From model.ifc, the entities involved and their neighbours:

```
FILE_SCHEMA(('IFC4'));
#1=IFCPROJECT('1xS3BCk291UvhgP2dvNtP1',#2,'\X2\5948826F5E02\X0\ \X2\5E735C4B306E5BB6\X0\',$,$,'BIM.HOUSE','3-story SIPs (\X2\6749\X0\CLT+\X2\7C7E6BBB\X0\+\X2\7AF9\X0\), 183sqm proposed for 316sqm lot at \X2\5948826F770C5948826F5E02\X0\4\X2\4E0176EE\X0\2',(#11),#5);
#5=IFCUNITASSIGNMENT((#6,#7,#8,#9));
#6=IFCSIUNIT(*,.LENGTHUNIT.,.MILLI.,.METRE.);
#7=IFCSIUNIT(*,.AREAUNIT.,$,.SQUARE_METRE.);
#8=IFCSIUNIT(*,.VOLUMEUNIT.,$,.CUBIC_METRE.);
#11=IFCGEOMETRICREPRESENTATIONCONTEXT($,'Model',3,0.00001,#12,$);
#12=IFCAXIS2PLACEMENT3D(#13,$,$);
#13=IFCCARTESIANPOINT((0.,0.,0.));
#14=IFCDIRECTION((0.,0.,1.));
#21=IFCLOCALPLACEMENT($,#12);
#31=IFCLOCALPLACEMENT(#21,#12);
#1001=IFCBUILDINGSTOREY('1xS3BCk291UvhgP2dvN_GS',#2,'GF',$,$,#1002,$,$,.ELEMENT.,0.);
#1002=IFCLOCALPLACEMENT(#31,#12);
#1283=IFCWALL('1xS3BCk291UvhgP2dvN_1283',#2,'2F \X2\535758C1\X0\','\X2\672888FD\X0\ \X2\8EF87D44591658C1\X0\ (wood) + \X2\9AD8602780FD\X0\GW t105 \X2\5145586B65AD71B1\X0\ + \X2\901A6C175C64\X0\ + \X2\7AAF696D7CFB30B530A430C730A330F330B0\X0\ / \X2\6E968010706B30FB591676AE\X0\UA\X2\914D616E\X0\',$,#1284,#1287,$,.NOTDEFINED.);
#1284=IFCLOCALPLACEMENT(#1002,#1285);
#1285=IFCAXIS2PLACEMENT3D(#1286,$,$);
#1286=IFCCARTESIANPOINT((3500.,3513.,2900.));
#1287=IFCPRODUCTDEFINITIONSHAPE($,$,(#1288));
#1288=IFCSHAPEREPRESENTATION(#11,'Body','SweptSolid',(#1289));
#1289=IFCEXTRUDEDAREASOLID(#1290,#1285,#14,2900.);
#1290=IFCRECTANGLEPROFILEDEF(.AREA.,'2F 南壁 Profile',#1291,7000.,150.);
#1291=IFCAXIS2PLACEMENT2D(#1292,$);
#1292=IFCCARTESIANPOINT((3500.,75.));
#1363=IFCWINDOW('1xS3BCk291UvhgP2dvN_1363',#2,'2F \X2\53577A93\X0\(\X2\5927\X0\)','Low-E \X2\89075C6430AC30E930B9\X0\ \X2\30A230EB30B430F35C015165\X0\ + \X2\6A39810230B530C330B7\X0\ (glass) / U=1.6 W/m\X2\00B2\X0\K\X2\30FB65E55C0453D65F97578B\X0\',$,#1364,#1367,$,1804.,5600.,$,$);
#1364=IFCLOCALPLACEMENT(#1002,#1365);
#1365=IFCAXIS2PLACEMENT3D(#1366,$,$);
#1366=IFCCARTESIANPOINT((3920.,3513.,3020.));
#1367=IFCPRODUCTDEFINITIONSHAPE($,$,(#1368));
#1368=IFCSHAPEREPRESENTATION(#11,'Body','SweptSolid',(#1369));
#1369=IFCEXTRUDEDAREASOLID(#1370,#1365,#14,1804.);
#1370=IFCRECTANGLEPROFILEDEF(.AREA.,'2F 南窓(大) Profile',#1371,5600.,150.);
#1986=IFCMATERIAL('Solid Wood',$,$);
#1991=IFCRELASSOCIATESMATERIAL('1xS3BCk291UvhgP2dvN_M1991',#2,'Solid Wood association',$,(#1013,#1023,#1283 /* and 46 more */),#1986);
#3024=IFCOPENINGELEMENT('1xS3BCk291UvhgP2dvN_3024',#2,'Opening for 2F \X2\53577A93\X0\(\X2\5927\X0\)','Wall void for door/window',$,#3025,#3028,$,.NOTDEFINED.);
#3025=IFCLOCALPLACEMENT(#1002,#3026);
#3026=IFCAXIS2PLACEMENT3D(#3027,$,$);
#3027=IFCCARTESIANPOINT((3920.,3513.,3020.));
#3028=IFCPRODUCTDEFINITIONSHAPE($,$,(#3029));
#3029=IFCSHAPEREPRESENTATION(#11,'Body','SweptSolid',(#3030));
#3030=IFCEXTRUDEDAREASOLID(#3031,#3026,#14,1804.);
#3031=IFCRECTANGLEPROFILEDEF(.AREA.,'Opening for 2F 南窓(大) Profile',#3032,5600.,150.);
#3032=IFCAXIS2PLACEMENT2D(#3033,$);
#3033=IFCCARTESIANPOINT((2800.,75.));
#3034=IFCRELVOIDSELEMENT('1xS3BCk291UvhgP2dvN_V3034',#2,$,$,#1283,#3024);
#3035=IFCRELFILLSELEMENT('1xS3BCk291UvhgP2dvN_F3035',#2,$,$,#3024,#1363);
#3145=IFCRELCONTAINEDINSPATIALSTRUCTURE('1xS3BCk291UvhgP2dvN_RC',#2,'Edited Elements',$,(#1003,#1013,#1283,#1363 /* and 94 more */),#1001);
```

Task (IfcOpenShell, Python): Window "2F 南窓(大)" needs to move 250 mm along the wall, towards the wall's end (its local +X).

```python
import ifcopenshell
import ifcopenshell.api.geometry
import ifcopenshell.util.placement
import ifcopenshell.util.unit

model = ifcopenshell.open("model.ifc")
unit_scale = ifcopenshell.util.unit.calculate_unit_scale(model)

window = model.by_guid("1xS3BCk291UvhgP2dvN_1363")
opening = window.FillsVoids[0].RelatingOpeningElement
wall = opening.VoidsElements[0].RelatingBuildingElement

wall_matrix = ifcopenshell.util.placement.get_local_placement(wall.ObjectPlacement)
shift = wall_matrix[:3, 0] * 0.25 / unit_scale
before = ifcopenshell.util.placement.get_local_placement(window.ObjectPlacement)[:3, 3].copy()

# The window is not placed relative to its opening, so move both.
for product in (opening, window):
    matrix = ifcopenshell.util.placement.get_local_placement(product.ObjectPlacement)
    matrix[:3, 3] += shift
    ifcopenshell.api.geometry.edit_object_placement(model, product=product, matrix=matrix, is_si=False)

after = ifcopenshell.util.placement.get_local_placement(window.ObjectPlacement)[:3, 3]
print("window moved by", (after - before).round(3) + 0.0)

model.write("model_rev.ifc")
```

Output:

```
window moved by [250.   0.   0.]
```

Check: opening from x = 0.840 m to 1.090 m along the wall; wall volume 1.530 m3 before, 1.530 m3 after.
